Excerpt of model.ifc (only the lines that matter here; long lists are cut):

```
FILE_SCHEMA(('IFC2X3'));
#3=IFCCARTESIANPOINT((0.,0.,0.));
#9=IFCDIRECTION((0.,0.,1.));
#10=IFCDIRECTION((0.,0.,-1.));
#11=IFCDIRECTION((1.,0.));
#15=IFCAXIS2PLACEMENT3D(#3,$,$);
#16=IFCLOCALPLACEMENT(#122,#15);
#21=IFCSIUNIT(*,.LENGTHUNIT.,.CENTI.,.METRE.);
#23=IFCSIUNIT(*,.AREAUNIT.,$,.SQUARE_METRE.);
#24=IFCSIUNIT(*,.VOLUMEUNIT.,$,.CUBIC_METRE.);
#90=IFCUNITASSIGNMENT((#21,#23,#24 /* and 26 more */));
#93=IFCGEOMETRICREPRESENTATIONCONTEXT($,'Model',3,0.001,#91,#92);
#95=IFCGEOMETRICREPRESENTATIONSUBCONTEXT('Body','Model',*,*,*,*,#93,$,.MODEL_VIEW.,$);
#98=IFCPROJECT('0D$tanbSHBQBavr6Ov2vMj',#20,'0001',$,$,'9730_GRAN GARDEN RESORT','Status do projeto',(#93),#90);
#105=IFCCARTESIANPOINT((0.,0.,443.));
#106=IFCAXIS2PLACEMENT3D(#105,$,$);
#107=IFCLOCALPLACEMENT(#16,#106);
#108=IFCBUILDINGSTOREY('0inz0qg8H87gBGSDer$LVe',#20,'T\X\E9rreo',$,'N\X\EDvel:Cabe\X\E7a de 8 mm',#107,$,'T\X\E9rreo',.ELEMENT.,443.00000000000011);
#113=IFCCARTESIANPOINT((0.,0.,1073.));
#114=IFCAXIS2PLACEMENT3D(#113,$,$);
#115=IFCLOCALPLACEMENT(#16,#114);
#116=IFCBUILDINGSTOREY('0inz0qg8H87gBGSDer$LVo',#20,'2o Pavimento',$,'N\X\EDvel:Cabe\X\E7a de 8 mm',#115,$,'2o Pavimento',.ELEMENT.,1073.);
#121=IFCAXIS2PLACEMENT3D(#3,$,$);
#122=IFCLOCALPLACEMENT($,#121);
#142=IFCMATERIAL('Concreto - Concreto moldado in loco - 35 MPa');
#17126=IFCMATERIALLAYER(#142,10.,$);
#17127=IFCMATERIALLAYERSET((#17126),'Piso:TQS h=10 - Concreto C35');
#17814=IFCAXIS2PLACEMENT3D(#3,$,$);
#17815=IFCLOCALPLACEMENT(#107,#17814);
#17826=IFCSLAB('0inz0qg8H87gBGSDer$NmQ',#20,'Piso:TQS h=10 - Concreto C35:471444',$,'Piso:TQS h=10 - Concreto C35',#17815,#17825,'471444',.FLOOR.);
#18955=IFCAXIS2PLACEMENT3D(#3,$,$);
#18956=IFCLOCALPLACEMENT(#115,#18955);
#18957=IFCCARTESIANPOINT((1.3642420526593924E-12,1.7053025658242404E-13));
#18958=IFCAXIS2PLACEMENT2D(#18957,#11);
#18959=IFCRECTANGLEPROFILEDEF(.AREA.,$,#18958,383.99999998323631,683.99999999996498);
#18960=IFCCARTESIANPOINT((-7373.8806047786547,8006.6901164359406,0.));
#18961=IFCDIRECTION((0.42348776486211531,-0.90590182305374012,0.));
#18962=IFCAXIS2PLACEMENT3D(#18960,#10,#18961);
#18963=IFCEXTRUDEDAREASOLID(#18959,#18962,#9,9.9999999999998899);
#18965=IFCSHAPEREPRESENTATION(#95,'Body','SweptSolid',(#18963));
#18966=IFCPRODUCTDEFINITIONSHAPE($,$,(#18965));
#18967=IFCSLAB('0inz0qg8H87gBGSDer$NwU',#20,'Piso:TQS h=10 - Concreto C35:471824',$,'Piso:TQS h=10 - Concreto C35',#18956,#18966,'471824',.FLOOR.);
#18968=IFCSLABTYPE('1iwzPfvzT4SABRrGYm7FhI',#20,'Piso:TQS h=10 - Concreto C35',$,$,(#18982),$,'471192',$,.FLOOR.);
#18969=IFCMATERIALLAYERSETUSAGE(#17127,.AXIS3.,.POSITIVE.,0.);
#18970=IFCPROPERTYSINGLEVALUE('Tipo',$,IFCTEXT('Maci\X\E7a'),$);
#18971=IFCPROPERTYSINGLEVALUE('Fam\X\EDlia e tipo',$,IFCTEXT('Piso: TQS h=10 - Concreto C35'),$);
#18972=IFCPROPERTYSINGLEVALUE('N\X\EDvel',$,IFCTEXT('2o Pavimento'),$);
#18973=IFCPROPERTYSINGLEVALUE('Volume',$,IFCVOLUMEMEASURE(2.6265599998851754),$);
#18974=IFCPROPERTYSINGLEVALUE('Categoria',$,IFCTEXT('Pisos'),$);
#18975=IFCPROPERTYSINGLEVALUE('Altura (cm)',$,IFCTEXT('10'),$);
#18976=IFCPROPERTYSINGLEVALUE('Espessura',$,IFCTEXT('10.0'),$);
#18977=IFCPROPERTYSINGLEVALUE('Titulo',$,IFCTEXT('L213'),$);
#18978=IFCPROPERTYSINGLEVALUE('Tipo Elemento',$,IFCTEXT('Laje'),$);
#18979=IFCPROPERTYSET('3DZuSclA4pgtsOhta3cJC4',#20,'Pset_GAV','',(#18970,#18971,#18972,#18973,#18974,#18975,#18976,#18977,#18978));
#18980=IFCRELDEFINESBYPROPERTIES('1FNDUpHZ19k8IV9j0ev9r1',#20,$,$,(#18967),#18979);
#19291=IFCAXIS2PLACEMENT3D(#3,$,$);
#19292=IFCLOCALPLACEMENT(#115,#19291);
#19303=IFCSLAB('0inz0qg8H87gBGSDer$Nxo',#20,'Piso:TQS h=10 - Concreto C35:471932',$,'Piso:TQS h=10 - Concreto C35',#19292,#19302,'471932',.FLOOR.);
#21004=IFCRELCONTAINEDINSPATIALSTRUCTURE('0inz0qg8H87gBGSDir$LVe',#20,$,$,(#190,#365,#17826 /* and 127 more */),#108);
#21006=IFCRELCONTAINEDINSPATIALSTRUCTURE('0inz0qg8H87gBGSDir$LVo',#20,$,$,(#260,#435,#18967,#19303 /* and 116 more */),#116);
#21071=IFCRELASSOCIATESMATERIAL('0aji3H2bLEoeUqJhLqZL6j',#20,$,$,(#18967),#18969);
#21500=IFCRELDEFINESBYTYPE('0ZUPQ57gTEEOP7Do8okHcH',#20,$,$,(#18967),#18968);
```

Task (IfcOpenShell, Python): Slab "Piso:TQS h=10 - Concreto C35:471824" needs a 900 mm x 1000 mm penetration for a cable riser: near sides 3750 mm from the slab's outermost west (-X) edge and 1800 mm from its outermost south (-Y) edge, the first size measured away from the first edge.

```python
import numpy as np
import ifcopenshell
import ifcopenshell.api.feature
import ifcopenshell.api.geometry
import ifcopenshell.api.pset
import ifcopenshell.api.root
import ifcopenshell.geom
import ifcopenshell.util.element
import ifcopenshell.util.placement
import ifcopenshell.util.representation
import ifcopenshell.util.shape
import ifcopenshell.util.unit

model = ifcopenshell.open("model.ifc")
unit_scale = ifcopenshell.util.unit.calculate_unit_scale(model)
volume_scale = ifcopenshell.util.unit.calculate_unit_scale(model, "VOLUMEUNIT")
settings = ifcopenshell.geom.settings()


def volume(element):
    """Net volume in cubic metres, openings subtracted."""
    shape = ifcopenshell.geom.create_shape(settings, element)
    return ifcopenshell.util.shape.get_volume(shape.geometry)


slab = model.by_guid("0inz0qg8H87gBGSDer$NwU")
before = volume(slab)

# Extent in the slab's own axes, in metres. The edges named are its -X and -Y sides.
slab_shape = ifcopenshell.geom.create_shape(settings, slab)
vertices = ifcopenshell.util.shape.get_vertices(slab_shape.geometry)
x_min, y_min, bottom = vertices.min(axis=0)
top = vertices[:, 2].max()

opening = ifcopenshell.api.root.create_entity(model, ifc_class="IfcOpeningElement", name="Cable riser opening")
context = ifcopenshell.util.representation.get_context(model, "Model", "Body", "MODEL_VIEW")
width, depth = 0.9, 1
outline = [(0.0, 0.0), (width, 0.0), (width, depth), (0.0, depth), (0.0, 0.0)]
# Overshoot both faces by 50 mm so the cut is clean.
shape = ifcopenshell.api.geometry.add_slab_representation(
    model, context=context, depth=top - bottom + 0.1, polyline=outline
)
ifcopenshell.api.geometry.assign_representation(model, product=opening, representation=shape)

matrix = ifcopenshell.util.placement.get_local_placement(slab.ObjectPlacement)
matrix[:, 3] = matrix @ np.append(np.array([x_min + 3.75, y_min + 1.8, bottom - 0.05]) / unit_scale, 1.0)
ifcopenshell.api.geometry.edit_object_placement(model, product=opening, matrix=matrix, is_si=False)
ifcopenshell.api.feature.add_feature(model, feature=opening, element=slab)

after = volume(slab)

# Update the slab's stored quantities.
pset = model.by_id(ifcopenshell.util.element.get_pset(slab, "Pset_GAV", should_inherit=False)["id"])
ifcopenshell.api.pset.edit_pset(model, pset=pset, properties={
    "Volume": model.create_entity("IfcVolumeMeasure", after / volume_scale),
})

print(f"slab volume {before:.3f} -> {after:.3f} m3")

model.write("model_edited.ifc")
```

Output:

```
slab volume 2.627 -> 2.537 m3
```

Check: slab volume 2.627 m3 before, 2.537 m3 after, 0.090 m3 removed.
